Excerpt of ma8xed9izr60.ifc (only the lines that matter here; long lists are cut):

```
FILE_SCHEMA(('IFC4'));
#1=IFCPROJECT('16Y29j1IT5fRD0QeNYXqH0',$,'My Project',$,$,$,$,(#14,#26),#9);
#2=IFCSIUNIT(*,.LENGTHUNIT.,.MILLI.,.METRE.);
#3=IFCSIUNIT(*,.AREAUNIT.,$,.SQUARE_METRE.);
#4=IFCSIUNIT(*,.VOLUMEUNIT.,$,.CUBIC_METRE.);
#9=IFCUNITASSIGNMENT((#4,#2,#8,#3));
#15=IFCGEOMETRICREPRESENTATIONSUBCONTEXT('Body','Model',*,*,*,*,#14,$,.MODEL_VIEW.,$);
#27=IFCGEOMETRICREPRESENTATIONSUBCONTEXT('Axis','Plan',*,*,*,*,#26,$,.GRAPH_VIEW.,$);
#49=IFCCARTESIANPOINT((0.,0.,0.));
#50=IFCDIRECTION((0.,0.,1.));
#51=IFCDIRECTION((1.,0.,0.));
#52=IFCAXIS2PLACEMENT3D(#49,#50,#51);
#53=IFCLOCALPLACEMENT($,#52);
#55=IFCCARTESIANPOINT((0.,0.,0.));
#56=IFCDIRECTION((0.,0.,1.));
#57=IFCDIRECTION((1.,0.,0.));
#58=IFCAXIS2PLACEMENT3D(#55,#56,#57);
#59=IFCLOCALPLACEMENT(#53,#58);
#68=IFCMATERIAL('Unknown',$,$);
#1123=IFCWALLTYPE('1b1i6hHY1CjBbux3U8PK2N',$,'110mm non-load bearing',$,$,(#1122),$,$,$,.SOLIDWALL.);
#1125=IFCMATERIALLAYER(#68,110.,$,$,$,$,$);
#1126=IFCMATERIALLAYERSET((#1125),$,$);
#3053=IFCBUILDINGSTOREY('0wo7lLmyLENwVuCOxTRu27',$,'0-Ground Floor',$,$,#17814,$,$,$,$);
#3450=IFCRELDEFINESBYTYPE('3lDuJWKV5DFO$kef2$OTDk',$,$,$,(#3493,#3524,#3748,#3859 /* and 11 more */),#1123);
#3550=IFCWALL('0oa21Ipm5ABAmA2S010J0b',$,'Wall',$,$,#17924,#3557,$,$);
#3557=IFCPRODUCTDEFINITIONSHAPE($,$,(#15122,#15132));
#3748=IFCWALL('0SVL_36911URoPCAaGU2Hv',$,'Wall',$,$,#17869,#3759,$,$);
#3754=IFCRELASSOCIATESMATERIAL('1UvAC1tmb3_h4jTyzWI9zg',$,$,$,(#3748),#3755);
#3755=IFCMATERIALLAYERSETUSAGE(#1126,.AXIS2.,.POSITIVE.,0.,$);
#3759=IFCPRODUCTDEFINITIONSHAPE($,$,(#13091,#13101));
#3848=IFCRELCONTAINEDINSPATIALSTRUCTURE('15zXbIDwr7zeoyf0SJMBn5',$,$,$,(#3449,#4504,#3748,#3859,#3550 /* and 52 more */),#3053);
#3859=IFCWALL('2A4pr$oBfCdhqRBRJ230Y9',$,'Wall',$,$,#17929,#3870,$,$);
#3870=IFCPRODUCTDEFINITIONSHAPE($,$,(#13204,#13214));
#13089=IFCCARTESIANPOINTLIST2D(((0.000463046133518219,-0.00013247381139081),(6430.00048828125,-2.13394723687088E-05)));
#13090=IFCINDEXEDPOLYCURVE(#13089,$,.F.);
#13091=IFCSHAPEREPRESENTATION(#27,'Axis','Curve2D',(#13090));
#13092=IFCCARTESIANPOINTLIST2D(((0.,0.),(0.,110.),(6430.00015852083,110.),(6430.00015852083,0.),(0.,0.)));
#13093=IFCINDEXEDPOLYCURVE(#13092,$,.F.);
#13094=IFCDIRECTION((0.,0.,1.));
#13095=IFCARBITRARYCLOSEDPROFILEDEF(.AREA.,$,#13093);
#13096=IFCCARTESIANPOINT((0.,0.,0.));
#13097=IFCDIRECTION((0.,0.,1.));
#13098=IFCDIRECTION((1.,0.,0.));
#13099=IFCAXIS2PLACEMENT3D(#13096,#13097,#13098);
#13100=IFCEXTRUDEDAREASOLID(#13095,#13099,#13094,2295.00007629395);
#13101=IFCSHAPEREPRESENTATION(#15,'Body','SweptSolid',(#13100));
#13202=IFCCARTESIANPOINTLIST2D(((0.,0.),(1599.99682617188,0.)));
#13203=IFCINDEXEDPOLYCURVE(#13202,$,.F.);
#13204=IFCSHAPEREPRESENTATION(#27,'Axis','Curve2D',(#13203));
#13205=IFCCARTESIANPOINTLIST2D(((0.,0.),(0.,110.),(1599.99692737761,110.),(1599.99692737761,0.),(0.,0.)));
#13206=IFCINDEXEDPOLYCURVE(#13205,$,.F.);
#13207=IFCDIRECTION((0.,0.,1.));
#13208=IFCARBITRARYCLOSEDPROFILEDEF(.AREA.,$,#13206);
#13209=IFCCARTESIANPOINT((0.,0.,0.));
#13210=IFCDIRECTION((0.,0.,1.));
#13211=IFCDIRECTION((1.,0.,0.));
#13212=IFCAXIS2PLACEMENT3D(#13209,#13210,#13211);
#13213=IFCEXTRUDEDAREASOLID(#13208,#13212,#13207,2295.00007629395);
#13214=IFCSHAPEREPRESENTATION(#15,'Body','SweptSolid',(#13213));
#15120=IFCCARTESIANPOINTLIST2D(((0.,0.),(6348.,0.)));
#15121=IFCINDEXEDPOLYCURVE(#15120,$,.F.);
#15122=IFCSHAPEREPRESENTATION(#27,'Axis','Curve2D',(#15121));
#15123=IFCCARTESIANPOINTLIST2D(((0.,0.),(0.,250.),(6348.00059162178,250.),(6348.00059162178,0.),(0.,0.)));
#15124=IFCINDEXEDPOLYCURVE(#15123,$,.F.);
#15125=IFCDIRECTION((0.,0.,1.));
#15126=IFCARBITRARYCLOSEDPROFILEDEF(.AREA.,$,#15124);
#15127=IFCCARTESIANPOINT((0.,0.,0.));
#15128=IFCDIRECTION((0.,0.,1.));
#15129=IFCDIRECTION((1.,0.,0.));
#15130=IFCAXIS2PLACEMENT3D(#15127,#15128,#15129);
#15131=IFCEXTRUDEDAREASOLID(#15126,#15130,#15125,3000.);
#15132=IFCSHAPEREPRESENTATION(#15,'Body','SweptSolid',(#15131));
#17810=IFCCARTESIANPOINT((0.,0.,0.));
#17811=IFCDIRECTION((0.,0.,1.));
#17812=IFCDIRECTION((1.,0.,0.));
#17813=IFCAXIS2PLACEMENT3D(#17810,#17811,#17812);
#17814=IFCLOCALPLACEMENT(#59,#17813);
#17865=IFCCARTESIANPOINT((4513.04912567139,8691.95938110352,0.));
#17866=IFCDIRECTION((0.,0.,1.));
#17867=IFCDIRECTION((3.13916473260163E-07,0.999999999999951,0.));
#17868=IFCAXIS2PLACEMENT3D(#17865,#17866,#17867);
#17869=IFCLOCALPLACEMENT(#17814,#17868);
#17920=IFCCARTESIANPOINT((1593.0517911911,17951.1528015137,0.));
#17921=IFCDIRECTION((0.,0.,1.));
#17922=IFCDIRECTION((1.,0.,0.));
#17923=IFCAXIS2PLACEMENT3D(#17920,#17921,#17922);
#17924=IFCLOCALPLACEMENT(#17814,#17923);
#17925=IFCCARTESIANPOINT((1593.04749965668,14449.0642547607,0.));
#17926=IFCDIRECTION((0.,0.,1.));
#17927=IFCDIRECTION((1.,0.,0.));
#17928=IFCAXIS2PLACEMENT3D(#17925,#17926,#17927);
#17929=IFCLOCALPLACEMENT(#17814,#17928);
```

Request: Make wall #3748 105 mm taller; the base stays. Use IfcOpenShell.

```python
import ifcopenshell
import ifcopenshell.geom
import ifcopenshell.util.representation
import ifcopenshell.util.shape

model = ifcopenshell.open("ma8xed9izr60.ifc")
settings = ifcopenshell.geom.settings()


def volume(element):
    """Net volume in cubic metres, openings subtracted."""
    shape = ifcopenshell.geom.create_shape(settings, element)
    return ifcopenshell.util.shape.get_volume(shape.geometry)


wall = model.by_guid("0SVL_36911URoPCAaGU2Hv")
before = volume(wall)

body = ifcopenshell.util.representation.get_representation(wall, "Model", "Body")
solid = body.Items[0]
old_height = solid.Depth
solid.Depth += 105.0
after = volume(wall)

print(f"height {old_height:g} -> {solid.Depth:g}, volume {before:.3f} -> {after:.3f} m3")

model.write("ma8xed9izr60_edited.ifc")
```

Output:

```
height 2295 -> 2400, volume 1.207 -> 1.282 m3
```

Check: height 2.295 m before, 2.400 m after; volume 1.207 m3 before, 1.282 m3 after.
